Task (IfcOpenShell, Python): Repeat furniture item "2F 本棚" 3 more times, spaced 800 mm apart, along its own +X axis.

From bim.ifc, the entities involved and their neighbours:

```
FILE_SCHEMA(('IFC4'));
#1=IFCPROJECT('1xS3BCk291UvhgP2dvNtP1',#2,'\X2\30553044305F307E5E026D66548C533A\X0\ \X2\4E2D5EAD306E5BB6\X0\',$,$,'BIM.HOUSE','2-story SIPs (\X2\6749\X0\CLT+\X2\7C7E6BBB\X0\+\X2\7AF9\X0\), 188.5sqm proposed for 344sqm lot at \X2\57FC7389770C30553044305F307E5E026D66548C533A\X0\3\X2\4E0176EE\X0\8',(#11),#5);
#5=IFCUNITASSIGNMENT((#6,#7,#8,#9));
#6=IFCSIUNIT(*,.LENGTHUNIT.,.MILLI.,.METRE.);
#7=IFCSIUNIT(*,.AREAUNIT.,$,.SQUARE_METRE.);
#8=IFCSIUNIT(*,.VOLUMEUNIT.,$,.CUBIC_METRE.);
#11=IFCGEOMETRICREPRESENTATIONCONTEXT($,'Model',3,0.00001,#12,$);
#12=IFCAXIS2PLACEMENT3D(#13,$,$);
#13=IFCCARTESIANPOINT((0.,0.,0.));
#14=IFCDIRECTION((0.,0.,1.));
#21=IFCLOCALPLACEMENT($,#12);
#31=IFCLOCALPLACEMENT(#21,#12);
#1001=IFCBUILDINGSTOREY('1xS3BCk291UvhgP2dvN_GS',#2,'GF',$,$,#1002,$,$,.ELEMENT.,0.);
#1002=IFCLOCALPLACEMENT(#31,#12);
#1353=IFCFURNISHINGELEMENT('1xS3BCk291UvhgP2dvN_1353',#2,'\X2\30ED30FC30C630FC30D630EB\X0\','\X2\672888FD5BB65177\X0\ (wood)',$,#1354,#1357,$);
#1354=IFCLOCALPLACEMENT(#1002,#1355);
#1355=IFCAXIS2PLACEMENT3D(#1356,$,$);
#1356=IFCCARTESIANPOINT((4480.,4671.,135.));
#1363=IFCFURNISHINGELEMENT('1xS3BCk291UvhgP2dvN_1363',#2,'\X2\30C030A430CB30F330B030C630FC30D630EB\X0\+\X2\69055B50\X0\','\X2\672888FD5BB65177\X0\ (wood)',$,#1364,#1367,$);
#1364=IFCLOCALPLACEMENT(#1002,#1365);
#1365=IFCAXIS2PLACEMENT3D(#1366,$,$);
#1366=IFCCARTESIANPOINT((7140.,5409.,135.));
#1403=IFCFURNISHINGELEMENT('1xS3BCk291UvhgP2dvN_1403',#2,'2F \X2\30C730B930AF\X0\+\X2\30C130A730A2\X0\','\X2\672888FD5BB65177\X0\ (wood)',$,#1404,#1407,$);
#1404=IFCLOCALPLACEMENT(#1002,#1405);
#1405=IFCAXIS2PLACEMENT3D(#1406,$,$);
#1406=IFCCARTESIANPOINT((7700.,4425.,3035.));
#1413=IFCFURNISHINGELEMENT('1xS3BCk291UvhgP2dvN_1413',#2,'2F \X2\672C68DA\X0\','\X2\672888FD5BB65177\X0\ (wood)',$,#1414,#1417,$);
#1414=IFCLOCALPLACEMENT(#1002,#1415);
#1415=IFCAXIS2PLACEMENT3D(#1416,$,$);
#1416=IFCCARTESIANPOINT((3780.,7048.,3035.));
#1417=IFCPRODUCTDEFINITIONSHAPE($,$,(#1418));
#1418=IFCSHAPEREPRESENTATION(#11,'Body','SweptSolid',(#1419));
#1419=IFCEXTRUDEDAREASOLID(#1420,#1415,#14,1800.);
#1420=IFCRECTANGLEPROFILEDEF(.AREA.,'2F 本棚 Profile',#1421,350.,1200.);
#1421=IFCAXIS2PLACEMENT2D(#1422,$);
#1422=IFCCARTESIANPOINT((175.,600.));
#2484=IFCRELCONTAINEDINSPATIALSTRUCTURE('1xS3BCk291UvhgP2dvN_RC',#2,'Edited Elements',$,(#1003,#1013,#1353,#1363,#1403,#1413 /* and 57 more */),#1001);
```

```python
import ifcopenshell
import ifcopenshell.api.geometry
import ifcopenshell.api.root
import ifcopenshell.util.element
import ifcopenshell.util.placement
import ifcopenshell.util.unit

model = ifcopenshell.open("bim.ifc")
unit_scale = ifcopenshell.util.unit.calculate_unit_scale(model)


def reuse_history(source, copy):
    """copy_class also copies each property set's owner history, people and application; keep the originals."""
    for rel in copy.IsDefinedBy:
        if rel.is_a("IfcRelDefinesByProperties") and (history := rel.RelatingPropertyDefinition.OwnerHistory):
            rel.RelatingPropertyDefinition.OwnerHistory = source.OwnerHistory
            ifcopenshell.util.element.remove_deep2(model, history)


source = model.by_guid("1xS3BCk291UvhgP2dvN_1413")
base = ifcopenshell.util.placement.get_local_placement(source.ObjectPlacement)
step = base[:3, 0] * 0.8 / unit_scale

for i in range(1, 4):
    copy = ifcopenshell.api.root.copy_class(model, product=source)
    copy.Representation = ifcopenshell.util.element.copy_deep(
        model, source.Representation, exclude=["IfcGeometricRepresentationContext", "IfcRepresentationMap"]
    )
    reuse_history(source, copy)
    matrix = base.copy()
    matrix[:3, 3] += i * step
    print("added at", matrix[:3, 3].round(3) + 0.0)
    ifcopenshell.api.geometry.edit_object_placement(model, product=copy, matrix=matrix, is_si=False)

model.write("bim_updated.ifc")
```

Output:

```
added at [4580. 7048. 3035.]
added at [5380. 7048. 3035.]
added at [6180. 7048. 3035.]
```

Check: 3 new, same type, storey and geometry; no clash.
